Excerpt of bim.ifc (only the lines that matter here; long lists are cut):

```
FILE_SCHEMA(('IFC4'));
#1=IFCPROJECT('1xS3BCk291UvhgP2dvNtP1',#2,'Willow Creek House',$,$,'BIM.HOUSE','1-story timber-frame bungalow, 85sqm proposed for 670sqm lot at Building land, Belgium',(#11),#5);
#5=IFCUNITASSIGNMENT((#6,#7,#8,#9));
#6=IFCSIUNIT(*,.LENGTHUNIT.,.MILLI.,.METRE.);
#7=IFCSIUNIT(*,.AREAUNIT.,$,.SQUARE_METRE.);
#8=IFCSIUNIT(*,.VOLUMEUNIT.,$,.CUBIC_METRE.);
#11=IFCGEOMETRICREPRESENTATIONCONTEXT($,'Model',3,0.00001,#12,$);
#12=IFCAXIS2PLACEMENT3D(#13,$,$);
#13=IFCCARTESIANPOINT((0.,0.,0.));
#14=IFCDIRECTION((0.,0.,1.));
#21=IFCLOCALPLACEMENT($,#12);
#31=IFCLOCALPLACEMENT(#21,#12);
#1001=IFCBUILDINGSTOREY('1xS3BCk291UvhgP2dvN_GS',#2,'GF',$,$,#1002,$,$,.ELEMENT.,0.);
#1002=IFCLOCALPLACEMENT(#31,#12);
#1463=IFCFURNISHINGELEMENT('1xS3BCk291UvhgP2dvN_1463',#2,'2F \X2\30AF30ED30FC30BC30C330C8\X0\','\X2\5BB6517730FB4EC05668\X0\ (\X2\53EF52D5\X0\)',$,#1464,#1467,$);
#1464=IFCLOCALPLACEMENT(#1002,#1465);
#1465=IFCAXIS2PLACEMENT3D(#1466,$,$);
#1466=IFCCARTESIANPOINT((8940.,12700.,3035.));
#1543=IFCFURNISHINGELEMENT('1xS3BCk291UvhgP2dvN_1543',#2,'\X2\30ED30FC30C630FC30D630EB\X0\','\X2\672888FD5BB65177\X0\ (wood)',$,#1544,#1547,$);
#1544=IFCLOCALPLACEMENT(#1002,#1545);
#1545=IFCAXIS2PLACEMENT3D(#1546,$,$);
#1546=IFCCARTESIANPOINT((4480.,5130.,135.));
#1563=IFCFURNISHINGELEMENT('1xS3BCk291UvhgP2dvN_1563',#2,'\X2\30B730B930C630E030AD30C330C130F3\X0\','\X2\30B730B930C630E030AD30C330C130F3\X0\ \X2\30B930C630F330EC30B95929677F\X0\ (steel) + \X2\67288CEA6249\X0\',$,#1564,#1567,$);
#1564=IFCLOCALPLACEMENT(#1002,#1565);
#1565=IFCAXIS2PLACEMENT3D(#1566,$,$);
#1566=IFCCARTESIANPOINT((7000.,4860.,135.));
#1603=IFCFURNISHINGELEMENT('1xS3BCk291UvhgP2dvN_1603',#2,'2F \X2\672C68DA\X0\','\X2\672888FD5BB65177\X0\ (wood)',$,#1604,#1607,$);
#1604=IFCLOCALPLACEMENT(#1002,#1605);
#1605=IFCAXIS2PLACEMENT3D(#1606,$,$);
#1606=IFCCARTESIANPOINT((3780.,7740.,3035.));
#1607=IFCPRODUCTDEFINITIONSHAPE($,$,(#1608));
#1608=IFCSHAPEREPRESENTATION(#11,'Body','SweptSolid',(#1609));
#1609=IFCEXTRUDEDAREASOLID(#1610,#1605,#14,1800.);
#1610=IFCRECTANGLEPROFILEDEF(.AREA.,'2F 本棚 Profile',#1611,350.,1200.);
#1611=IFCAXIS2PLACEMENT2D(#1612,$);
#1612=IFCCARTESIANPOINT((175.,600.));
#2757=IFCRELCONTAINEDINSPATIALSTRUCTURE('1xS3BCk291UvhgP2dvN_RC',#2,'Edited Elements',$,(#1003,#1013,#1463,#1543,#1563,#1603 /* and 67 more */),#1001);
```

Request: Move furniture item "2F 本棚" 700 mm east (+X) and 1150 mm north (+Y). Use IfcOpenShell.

```python
import ifcopenshell
import ifcopenshell.api.geometry
import ifcopenshell.util.placement

model = ifcopenshell.open("bim.ifc")

item = model.by_guid("1xS3BCk291UvhgP2dvN_1603")
matrix = ifcopenshell.util.placement.get_local_placement(item.ObjectPlacement)
matrix[0, 3] += 700.0
matrix[1, 3] += 1150.0
ifcopenshell.api.geometry.edit_object_placement(model, product=item, matrix=matrix, is_si=False)

print(ifcopenshell.util.placement.get_local_placement(item.ObjectPlacement).round(3) + 0.0)

model.write("bim-out.ifc")
```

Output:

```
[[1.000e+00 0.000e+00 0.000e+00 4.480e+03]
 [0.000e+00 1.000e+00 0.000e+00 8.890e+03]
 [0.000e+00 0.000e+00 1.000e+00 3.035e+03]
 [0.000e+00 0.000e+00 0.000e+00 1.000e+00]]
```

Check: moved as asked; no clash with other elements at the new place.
